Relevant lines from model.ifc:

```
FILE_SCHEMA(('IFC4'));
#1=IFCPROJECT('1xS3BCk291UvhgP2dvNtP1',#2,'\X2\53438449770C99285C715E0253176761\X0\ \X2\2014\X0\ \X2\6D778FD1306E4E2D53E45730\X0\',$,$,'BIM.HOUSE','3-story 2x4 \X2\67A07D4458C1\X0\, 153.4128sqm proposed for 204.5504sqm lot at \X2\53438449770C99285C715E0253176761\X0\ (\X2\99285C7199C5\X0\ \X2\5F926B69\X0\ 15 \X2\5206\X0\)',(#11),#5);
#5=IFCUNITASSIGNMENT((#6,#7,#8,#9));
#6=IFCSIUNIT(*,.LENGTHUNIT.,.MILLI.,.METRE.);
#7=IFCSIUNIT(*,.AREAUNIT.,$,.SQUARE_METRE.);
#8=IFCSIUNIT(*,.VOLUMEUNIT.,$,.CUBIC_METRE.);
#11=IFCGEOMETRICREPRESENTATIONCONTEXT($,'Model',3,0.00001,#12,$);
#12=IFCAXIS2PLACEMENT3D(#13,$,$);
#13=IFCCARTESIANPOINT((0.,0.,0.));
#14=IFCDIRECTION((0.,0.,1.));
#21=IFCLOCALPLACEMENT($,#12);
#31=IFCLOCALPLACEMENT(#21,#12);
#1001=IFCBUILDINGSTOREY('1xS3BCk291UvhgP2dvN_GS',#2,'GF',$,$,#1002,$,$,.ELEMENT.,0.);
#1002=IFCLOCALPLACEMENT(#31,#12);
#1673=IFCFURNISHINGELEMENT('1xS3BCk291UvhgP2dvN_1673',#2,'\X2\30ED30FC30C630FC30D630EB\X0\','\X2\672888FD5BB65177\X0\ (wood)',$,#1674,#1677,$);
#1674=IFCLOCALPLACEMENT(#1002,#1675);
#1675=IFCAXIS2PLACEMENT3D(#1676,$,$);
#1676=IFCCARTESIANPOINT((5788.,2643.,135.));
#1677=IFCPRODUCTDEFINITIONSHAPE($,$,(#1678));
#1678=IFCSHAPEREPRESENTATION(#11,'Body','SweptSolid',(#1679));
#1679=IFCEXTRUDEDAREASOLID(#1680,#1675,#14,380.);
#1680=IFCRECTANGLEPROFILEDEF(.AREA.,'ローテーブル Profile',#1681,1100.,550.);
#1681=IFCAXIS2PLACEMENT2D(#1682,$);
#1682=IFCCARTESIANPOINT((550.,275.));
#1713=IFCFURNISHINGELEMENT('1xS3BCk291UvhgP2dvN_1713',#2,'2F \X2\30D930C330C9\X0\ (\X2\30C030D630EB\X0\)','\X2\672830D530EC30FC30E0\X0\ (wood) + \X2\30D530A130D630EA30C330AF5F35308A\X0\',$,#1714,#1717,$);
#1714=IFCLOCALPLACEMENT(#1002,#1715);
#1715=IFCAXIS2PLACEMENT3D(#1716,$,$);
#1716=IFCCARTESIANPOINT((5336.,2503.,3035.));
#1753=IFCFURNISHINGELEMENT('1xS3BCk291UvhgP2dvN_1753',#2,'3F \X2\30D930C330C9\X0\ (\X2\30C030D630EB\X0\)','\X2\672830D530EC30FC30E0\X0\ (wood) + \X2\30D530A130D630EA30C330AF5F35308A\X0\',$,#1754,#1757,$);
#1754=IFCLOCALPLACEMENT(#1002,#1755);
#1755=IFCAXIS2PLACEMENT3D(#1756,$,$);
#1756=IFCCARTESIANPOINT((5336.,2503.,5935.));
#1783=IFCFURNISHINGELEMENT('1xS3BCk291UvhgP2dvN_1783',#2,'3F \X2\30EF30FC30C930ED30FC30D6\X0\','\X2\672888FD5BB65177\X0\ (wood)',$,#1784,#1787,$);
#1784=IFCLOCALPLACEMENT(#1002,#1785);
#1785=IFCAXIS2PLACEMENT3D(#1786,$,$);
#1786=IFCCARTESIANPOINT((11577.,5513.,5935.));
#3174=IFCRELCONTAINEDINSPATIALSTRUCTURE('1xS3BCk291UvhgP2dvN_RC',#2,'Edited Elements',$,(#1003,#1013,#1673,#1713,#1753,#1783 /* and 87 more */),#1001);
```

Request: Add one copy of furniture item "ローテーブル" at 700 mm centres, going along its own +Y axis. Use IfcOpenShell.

```python
import ifcopenshell
import ifcopenshell.api.geometry
import ifcopenshell.api.root
import ifcopenshell.util.element
import ifcopenshell.util.placement
import ifcopenshell.util.unit

model = ifcopenshell.open("model.ifc")
unit_scale = ifcopenshell.util.unit.calculate_unit_scale(model)


def reuse_history(source, copy):
    """copy_class also copies each property set's owner history, people and application; keep the originals."""
    for rel in copy.IsDefinedBy:
        if rel.is_a("IfcRelDefinesByProperties") and (history := rel.RelatingPropertyDefinition.OwnerHistory):
            rel.RelatingPropertyDefinition.OwnerHistory = source.OwnerHistory
            ifcopenshell.util.element.remove_deep2(model, history)


source = model.by_guid("1xS3BCk291UvhgP2dvN_1673")
base = ifcopenshell.util.placement.get_local_placement(source.ObjectPlacement)
step = base[:3, 1] * 0.7 / unit_scale

for i in range(1, 2):
    copy = ifcopenshell.api.root.copy_class(model, product=source)
    copy.Representation = ifcopenshell.util.element.copy_deep(
        model, source.Representation, exclude=["IfcGeometricRepresentationContext", "IfcRepresentationMap"]
    )
    reuse_history(source, copy)
    matrix = base.copy()
    matrix[:3, 3] += i * step
    print("added at", matrix[:3, 3].round(3) + 0.0)
    ifcopenshell.api.geometry.edit_object_placement(model, product=copy, matrix=matrix, is_si=False)

model.write("model_v2.ifc")
```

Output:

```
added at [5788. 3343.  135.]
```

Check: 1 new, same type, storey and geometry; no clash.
